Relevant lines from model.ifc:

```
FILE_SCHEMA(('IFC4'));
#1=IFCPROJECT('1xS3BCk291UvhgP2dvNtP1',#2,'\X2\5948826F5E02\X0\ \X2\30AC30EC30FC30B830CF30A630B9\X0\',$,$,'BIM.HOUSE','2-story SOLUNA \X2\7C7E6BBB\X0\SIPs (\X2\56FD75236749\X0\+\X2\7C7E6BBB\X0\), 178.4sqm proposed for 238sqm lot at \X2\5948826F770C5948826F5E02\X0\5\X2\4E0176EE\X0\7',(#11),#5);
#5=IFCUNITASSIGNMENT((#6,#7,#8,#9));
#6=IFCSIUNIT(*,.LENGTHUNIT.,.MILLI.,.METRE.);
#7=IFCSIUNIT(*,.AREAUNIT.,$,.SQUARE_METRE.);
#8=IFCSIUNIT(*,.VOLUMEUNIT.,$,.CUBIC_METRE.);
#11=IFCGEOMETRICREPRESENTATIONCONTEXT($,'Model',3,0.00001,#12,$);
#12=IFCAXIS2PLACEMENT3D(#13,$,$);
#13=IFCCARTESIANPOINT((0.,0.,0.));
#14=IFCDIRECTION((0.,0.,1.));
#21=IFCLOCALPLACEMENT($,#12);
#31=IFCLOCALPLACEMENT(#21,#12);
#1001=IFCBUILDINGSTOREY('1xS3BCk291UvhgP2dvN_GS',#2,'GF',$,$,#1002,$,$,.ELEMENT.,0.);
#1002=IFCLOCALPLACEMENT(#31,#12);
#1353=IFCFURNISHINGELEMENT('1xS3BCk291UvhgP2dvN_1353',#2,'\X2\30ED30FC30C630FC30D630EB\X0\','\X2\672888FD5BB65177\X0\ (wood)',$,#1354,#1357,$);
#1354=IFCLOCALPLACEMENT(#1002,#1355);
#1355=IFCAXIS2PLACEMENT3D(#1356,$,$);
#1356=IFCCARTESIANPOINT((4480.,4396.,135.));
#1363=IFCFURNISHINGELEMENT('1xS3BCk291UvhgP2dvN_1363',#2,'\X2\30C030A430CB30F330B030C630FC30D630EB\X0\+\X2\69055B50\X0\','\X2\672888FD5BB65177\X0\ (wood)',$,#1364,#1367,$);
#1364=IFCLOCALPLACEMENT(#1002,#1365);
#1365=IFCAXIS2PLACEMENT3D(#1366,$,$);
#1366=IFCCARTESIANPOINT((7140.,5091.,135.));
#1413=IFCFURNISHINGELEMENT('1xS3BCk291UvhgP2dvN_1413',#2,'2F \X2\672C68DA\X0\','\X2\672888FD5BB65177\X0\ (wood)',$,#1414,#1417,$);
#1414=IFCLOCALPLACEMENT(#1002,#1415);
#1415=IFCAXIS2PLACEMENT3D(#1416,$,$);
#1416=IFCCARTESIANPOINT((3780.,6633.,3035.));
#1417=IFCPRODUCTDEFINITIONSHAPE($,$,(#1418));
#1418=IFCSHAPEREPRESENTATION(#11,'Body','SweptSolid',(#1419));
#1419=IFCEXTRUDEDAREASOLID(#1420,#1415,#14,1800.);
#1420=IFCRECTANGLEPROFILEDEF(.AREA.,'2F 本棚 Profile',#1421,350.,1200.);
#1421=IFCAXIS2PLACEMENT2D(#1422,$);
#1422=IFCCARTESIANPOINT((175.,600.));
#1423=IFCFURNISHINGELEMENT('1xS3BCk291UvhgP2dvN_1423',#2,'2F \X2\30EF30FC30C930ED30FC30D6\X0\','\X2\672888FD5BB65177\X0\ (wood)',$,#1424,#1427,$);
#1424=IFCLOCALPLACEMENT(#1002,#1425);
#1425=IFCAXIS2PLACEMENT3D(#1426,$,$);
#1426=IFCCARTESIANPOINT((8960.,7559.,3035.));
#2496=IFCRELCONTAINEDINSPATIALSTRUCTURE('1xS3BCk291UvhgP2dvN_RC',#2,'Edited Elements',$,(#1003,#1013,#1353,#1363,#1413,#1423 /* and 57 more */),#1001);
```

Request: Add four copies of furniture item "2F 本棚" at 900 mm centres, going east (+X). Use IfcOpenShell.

```python
import numpy as np
import ifcopenshell
import ifcopenshell.api.geometry
import ifcopenshell.api.root
import ifcopenshell.util.element
import ifcopenshell.util.placement
import ifcopenshell.util.unit

model = ifcopenshell.open("model.ifc")
unit_scale = ifcopenshell.util.unit.calculate_unit_scale(model)


def reuse_history(source, copy):
    """copy_class also copies each property set's owner history, people and application; keep the originals."""
    for rel in copy.IsDefinedBy:
        if rel.is_a("IfcRelDefinesByProperties") and (history := rel.RelatingPropertyDefinition.OwnerHistory):
            rel.RelatingPropertyDefinition.OwnerHistory = source.OwnerHistory
            ifcopenshell.util.element.remove_deep2(model, history)


source = model.by_id(1413)
base = ifcopenshell.util.placement.get_local_placement(source.ObjectPlacement)
step = np.array([1.0, 0.0, 0.0]) * 0.9 / unit_scale

for i in range(1, 5):
    copy = ifcopenshell.api.root.copy_class(model, product=source)
    copy.Representation = ifcopenshell.util.element.copy_deep(
        model, source.Representation, exclude=["IfcGeometricRepresentationContext", "IfcRepresentationMap"]
    )
    reuse_history(source, copy)
    matrix = base.copy()
    matrix[:3, 3] += i * step
    print("added at", matrix[:3, 3].round(3) + 0.0)
    ifcopenshell.api.geometry.edit_object_placement(model, product=copy, matrix=matrix, is_si=False)

model.write("model-out.ifc")
```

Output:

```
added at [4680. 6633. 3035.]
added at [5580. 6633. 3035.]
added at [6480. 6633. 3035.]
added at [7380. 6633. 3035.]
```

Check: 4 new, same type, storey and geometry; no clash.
